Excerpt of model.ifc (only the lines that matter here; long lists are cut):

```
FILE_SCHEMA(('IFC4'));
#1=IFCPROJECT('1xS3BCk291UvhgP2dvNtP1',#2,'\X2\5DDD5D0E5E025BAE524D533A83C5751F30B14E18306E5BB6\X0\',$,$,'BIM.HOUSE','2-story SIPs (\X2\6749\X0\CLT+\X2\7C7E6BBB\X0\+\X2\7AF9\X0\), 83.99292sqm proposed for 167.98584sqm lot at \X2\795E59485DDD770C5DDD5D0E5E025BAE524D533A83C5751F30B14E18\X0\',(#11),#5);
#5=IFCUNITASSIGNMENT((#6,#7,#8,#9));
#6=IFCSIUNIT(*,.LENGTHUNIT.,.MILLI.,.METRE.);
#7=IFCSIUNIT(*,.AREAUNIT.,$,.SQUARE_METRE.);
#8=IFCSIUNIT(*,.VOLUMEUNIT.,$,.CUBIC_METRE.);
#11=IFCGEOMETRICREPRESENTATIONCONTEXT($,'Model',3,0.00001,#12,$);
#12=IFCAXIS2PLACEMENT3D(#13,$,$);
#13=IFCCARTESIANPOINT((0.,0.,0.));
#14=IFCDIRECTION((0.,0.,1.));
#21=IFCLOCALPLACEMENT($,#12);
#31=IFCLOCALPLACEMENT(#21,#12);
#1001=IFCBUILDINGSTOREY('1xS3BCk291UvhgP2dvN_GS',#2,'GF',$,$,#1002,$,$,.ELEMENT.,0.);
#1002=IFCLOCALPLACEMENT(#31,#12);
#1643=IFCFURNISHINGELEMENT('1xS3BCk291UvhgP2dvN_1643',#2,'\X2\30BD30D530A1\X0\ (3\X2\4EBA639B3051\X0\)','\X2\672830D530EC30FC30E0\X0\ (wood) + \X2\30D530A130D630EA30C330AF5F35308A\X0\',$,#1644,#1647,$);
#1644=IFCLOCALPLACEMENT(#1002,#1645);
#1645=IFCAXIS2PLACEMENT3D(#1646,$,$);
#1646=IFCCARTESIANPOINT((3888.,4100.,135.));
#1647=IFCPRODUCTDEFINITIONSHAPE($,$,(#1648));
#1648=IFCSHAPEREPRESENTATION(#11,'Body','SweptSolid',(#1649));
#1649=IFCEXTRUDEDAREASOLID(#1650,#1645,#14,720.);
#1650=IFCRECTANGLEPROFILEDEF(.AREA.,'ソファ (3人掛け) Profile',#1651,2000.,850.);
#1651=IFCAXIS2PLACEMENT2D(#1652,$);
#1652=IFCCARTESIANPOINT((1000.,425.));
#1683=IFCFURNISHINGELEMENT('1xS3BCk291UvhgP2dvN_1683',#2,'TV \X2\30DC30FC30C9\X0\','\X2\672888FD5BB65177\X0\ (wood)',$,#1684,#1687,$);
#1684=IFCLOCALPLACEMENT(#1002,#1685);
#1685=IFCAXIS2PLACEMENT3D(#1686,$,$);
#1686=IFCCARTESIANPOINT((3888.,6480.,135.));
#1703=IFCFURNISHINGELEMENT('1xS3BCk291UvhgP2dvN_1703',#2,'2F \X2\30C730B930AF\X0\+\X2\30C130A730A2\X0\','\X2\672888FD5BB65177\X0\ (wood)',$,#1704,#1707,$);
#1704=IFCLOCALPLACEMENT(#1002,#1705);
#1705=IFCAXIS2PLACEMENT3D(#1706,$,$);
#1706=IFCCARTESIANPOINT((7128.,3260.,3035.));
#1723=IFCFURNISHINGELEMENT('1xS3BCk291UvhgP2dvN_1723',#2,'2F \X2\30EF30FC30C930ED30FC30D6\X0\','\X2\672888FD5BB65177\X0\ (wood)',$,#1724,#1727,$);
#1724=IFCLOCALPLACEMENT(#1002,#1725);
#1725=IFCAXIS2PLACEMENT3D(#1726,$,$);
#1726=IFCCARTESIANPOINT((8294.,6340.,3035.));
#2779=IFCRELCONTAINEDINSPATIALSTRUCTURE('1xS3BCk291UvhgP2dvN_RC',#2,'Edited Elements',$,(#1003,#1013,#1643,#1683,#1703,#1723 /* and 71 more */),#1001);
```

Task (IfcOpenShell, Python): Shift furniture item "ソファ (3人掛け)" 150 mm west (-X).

```python
import ifcopenshell
import ifcopenshell.api.geometry
import ifcopenshell.util.placement
import ifcopenshell.util.unit

model = ifcopenshell.open("model.ifc")
unit_scale = ifcopenshell.util.unit.calculate_unit_scale(model)

item = model.by_guid("1xS3BCk291UvhgP2dvN_1643")
matrix = ifcopenshell.util.placement.get_local_placement(item.ObjectPlacement)
matrix[0, 3] -= 0.15 / unit_scale
ifcopenshell.api.geometry.edit_object_placement(model, product=item, matrix=matrix, is_si=False)

print(ifcopenshell.util.placement.get_local_placement(item.ObjectPlacement).round(3) + 0.0)

model.write("model_updated.ifc")
```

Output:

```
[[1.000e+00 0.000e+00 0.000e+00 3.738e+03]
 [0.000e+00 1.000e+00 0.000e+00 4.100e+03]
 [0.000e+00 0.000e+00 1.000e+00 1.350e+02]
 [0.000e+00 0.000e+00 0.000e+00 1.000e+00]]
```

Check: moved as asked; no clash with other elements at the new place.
